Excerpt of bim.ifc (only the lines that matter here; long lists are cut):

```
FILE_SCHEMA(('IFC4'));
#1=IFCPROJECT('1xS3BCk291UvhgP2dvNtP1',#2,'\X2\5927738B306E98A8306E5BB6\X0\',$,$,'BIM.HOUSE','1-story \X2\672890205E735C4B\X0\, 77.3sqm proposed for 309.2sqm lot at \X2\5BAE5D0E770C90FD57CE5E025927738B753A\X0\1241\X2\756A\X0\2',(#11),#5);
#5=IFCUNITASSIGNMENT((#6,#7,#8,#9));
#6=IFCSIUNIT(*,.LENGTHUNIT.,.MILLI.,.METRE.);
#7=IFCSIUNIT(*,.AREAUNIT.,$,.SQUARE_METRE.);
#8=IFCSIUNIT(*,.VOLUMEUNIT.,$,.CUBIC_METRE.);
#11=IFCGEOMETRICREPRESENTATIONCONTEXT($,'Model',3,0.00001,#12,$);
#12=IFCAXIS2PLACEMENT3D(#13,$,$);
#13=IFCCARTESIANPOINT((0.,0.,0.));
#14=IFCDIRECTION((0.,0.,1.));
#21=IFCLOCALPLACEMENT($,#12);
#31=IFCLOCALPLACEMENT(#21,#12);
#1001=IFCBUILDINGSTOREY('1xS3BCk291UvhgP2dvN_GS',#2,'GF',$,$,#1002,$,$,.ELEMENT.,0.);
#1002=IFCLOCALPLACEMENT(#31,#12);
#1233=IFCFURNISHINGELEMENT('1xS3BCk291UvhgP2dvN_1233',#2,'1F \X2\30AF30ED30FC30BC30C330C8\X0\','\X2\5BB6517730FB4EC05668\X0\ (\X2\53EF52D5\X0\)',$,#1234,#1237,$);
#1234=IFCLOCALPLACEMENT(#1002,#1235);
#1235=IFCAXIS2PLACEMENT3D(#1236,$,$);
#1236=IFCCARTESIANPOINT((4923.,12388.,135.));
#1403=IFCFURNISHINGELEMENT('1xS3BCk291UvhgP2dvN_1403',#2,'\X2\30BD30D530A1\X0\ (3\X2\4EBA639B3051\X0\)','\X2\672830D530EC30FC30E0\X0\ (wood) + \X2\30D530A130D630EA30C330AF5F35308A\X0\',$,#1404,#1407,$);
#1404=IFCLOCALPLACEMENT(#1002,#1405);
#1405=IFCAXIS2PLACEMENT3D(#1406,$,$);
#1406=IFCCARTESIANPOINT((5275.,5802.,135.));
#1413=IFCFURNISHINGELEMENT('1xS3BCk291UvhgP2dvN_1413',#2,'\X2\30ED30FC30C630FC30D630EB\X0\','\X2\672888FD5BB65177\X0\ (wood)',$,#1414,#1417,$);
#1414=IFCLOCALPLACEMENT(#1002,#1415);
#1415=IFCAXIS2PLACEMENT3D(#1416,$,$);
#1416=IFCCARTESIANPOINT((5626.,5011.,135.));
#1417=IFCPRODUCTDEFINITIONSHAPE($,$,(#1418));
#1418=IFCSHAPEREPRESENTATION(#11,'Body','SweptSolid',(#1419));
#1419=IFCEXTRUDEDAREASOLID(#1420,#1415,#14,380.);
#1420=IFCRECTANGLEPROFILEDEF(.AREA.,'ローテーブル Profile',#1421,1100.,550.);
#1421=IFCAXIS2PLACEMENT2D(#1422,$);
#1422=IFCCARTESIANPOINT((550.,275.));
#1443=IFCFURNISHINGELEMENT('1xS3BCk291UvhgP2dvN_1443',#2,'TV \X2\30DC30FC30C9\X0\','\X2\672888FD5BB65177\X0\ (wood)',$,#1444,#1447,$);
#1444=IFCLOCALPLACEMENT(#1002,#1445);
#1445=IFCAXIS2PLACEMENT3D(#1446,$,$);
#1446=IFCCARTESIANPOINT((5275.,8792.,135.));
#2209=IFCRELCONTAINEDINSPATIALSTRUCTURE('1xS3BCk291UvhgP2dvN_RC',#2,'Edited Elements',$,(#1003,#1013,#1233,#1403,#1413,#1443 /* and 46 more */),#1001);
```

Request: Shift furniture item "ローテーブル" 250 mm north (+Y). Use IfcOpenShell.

```python
import ifcopenshell
import ifcopenshell.api.geometry
import ifcopenshell.util.placement
import ifcopenshell.util.unit

model = ifcopenshell.open("bim.ifc")
unit_scale = ifcopenshell.util.unit.calculate_unit_scale(model)

item = model.by_guid("1xS3BCk291UvhgP2dvN_1413")
matrix = ifcopenshell.util.placement.get_local_placement(item.ObjectPlacement)
matrix[1, 3] += 0.25 / unit_scale
ifcopenshell.api.geometry.edit_object_placement(model, product=item, matrix=matrix, is_si=False)

print(ifcopenshell.util.placement.get_local_placement(item.ObjectPlacement).round(3) + 0.0)

model.write("bim_rev.ifc")
```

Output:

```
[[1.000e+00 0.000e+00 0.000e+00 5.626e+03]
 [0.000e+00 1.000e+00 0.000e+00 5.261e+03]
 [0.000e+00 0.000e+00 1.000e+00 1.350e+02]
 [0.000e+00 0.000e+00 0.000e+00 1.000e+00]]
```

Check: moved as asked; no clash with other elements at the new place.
